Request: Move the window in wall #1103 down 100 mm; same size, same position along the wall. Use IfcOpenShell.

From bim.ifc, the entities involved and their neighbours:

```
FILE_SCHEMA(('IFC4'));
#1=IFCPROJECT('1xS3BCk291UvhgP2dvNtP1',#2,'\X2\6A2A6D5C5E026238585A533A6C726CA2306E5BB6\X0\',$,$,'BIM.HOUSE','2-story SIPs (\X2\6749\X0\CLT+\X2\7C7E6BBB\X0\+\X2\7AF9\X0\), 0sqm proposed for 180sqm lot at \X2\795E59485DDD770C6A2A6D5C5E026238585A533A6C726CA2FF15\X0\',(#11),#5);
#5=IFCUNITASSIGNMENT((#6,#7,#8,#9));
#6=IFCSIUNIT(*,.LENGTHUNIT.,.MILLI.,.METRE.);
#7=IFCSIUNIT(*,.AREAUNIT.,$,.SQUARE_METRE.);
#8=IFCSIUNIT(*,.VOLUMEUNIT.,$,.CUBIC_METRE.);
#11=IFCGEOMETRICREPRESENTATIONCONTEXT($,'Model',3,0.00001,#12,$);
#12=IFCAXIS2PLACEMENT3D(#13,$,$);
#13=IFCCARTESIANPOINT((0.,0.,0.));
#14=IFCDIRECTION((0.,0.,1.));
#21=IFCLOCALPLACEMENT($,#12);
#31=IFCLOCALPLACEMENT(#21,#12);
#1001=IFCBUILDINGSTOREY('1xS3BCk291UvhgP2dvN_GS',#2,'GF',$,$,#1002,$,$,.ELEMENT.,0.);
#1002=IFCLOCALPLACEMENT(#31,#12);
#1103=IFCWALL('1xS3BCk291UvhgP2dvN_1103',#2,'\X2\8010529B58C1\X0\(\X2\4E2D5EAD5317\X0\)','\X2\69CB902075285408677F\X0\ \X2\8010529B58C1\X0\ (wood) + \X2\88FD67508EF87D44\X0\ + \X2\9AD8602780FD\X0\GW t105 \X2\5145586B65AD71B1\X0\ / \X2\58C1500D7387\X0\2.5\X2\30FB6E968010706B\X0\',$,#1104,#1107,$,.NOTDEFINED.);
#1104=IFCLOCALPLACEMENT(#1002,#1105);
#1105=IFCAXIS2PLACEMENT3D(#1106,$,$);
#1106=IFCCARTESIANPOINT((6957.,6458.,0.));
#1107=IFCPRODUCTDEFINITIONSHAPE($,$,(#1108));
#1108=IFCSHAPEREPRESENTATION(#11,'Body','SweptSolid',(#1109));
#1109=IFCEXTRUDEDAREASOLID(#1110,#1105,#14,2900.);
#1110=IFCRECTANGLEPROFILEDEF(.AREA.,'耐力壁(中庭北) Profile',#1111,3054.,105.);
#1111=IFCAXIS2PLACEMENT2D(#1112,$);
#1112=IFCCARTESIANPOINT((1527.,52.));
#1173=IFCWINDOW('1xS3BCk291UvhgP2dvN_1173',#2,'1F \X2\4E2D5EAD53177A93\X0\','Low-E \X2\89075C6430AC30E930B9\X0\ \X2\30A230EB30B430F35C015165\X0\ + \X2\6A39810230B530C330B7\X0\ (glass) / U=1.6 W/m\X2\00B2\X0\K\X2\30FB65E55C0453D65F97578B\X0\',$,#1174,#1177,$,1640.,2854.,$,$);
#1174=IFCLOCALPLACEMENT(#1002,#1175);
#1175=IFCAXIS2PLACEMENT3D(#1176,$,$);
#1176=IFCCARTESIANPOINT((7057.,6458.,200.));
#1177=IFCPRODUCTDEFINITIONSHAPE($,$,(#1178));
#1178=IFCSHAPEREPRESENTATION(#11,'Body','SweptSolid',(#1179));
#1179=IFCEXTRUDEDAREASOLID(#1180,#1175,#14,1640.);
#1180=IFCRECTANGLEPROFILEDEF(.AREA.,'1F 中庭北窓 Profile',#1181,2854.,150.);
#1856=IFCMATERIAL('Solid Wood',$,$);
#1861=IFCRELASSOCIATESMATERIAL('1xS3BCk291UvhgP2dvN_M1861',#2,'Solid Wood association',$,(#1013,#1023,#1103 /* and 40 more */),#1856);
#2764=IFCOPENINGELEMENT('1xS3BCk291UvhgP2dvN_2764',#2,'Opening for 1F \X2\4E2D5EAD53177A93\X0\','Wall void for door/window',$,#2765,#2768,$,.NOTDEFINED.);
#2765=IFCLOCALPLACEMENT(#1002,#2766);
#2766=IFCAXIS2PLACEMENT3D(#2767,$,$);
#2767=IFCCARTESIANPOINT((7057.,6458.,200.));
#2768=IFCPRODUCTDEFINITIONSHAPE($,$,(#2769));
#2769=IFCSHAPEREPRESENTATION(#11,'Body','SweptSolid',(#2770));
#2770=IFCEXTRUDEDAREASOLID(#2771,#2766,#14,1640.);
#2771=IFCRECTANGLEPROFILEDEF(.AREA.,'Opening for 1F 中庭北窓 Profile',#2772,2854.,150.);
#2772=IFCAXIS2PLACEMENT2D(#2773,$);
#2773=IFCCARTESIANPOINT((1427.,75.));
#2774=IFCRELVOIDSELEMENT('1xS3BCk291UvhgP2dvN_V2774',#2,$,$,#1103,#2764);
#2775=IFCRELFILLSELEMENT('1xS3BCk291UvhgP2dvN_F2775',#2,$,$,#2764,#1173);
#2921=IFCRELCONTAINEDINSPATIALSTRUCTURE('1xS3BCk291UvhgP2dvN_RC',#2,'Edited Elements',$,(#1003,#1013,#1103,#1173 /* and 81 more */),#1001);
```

```python
import numpy as np
import ifcopenshell
import ifcopenshell.api.geometry
import ifcopenshell.util.placement
import ifcopenshell.util.unit

model = ifcopenshell.open("bim.ifc")
unit_scale = ifcopenshell.util.unit.calculate_unit_scale(model)

window = model.by_guid("1xS3BCk291UvhgP2dvN_1173")
opening = window.FillsVoids[0].RelatingOpeningElement
dz = -100.0

shift = np.array([0.0, 0.0, dz])
# The window is not placed relative to its opening, so move both.
for product in (opening, window):
    matrix = ifcopenshell.util.placement.get_local_placement(product.ObjectPlacement)
    matrix[:3, 3] += shift
    ifcopenshell.api.geometry.edit_object_placement(model, product=product, matrix=matrix, is_si=False)

print(f"moved by {dz * unit_scale:+.3f} m")

model.write("bim_updated.ifc")
```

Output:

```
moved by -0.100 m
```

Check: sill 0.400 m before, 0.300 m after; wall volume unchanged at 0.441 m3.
